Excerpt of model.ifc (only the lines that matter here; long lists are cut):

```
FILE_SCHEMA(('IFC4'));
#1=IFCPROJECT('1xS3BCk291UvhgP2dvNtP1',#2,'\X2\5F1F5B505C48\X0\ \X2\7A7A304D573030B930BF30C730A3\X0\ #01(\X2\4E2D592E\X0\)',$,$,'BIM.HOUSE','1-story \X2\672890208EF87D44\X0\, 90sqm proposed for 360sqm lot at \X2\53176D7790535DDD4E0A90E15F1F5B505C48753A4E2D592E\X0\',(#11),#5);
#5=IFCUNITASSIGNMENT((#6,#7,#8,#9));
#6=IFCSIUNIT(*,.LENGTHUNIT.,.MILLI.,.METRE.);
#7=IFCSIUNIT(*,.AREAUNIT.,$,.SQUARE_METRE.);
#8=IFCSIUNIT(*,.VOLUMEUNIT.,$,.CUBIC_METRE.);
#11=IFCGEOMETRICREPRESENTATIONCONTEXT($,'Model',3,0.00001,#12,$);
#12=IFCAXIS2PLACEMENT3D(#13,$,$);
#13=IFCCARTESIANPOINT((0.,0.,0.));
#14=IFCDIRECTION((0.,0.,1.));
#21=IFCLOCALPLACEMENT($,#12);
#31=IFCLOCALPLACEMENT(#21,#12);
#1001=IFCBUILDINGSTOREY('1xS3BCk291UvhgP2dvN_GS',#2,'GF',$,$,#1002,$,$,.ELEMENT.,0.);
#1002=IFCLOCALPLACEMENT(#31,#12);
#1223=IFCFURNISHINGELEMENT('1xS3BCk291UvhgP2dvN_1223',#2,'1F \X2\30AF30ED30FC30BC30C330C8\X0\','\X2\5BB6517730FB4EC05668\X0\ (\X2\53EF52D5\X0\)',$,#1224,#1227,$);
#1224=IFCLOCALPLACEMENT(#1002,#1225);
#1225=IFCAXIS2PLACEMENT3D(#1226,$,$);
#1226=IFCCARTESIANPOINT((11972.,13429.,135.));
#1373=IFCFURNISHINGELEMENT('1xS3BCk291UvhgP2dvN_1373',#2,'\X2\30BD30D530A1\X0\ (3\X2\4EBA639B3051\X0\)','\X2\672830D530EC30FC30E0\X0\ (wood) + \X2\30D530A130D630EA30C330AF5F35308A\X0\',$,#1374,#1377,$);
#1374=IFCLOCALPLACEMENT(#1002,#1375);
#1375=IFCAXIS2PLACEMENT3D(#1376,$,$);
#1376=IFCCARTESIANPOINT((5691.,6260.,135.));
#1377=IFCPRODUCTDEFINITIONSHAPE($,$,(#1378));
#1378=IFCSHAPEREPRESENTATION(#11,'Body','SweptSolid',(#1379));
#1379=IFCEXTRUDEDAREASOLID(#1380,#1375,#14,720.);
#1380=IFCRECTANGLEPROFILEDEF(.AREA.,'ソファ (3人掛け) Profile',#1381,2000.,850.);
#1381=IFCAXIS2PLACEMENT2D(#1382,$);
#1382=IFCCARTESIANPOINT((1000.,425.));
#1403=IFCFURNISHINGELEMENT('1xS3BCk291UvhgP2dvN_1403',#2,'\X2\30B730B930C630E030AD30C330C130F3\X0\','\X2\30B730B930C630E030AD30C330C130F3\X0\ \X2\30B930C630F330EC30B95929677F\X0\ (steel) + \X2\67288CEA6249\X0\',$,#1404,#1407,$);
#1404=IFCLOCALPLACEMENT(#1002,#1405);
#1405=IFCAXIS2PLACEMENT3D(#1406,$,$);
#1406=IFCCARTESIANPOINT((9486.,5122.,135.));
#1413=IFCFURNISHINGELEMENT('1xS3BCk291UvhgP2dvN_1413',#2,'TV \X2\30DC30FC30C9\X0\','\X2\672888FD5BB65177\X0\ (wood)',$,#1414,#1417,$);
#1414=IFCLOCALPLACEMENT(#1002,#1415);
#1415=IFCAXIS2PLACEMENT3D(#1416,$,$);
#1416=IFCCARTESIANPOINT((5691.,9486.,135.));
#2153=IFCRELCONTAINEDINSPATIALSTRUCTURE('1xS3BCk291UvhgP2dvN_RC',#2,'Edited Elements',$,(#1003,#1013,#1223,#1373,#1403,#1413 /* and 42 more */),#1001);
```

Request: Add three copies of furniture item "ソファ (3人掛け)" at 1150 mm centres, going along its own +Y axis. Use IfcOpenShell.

```python
import ifcopenshell
import ifcopenshell.api.geometry
import ifcopenshell.api.root
import ifcopenshell.util.element
import ifcopenshell.util.placement
import ifcopenshell.util.unit

model = ifcopenshell.open("model.ifc")
unit_scale = ifcopenshell.util.unit.calculate_unit_scale(model)


def reuse_history(source, copy):
    """copy_class also copies each property set's owner history, people and application; keep the originals."""
    for rel in copy.IsDefinedBy:
        if rel.is_a("IfcRelDefinesByProperties") and (history := rel.RelatingPropertyDefinition.OwnerHistory):
            rel.RelatingPropertyDefinition.OwnerHistory = source.OwnerHistory
            ifcopenshell.util.element.remove_deep2(model, history)


source = model.by_guid("1xS3BCk291UvhgP2dvN_1373")
base = ifcopenshell.util.placement.get_local_placement(source.ObjectPlacement)
step = base[:3, 1] * 1.15 / unit_scale

for i in range(1, 4):
    copy = ifcopenshell.api.root.copy_class(model, product=source)
    copy.Representation = ifcopenshell.util.element.copy_deep(
        model, source.Representation, exclude=["IfcGeometricRepresentationContext", "IfcRepresentationMap"]
    )
    reuse_history(source, copy)
    matrix = base.copy()
    matrix[:3, 3] += i * step
    print("added at", matrix[:3, 3].round(3) + 0.0)
    ifcopenshell.api.geometry.edit_object_placement(model, product=copy, matrix=matrix, is_si=False)

model.write("model-out.ifc")
```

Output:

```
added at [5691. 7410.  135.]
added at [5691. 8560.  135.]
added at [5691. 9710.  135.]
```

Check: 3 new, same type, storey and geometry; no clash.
